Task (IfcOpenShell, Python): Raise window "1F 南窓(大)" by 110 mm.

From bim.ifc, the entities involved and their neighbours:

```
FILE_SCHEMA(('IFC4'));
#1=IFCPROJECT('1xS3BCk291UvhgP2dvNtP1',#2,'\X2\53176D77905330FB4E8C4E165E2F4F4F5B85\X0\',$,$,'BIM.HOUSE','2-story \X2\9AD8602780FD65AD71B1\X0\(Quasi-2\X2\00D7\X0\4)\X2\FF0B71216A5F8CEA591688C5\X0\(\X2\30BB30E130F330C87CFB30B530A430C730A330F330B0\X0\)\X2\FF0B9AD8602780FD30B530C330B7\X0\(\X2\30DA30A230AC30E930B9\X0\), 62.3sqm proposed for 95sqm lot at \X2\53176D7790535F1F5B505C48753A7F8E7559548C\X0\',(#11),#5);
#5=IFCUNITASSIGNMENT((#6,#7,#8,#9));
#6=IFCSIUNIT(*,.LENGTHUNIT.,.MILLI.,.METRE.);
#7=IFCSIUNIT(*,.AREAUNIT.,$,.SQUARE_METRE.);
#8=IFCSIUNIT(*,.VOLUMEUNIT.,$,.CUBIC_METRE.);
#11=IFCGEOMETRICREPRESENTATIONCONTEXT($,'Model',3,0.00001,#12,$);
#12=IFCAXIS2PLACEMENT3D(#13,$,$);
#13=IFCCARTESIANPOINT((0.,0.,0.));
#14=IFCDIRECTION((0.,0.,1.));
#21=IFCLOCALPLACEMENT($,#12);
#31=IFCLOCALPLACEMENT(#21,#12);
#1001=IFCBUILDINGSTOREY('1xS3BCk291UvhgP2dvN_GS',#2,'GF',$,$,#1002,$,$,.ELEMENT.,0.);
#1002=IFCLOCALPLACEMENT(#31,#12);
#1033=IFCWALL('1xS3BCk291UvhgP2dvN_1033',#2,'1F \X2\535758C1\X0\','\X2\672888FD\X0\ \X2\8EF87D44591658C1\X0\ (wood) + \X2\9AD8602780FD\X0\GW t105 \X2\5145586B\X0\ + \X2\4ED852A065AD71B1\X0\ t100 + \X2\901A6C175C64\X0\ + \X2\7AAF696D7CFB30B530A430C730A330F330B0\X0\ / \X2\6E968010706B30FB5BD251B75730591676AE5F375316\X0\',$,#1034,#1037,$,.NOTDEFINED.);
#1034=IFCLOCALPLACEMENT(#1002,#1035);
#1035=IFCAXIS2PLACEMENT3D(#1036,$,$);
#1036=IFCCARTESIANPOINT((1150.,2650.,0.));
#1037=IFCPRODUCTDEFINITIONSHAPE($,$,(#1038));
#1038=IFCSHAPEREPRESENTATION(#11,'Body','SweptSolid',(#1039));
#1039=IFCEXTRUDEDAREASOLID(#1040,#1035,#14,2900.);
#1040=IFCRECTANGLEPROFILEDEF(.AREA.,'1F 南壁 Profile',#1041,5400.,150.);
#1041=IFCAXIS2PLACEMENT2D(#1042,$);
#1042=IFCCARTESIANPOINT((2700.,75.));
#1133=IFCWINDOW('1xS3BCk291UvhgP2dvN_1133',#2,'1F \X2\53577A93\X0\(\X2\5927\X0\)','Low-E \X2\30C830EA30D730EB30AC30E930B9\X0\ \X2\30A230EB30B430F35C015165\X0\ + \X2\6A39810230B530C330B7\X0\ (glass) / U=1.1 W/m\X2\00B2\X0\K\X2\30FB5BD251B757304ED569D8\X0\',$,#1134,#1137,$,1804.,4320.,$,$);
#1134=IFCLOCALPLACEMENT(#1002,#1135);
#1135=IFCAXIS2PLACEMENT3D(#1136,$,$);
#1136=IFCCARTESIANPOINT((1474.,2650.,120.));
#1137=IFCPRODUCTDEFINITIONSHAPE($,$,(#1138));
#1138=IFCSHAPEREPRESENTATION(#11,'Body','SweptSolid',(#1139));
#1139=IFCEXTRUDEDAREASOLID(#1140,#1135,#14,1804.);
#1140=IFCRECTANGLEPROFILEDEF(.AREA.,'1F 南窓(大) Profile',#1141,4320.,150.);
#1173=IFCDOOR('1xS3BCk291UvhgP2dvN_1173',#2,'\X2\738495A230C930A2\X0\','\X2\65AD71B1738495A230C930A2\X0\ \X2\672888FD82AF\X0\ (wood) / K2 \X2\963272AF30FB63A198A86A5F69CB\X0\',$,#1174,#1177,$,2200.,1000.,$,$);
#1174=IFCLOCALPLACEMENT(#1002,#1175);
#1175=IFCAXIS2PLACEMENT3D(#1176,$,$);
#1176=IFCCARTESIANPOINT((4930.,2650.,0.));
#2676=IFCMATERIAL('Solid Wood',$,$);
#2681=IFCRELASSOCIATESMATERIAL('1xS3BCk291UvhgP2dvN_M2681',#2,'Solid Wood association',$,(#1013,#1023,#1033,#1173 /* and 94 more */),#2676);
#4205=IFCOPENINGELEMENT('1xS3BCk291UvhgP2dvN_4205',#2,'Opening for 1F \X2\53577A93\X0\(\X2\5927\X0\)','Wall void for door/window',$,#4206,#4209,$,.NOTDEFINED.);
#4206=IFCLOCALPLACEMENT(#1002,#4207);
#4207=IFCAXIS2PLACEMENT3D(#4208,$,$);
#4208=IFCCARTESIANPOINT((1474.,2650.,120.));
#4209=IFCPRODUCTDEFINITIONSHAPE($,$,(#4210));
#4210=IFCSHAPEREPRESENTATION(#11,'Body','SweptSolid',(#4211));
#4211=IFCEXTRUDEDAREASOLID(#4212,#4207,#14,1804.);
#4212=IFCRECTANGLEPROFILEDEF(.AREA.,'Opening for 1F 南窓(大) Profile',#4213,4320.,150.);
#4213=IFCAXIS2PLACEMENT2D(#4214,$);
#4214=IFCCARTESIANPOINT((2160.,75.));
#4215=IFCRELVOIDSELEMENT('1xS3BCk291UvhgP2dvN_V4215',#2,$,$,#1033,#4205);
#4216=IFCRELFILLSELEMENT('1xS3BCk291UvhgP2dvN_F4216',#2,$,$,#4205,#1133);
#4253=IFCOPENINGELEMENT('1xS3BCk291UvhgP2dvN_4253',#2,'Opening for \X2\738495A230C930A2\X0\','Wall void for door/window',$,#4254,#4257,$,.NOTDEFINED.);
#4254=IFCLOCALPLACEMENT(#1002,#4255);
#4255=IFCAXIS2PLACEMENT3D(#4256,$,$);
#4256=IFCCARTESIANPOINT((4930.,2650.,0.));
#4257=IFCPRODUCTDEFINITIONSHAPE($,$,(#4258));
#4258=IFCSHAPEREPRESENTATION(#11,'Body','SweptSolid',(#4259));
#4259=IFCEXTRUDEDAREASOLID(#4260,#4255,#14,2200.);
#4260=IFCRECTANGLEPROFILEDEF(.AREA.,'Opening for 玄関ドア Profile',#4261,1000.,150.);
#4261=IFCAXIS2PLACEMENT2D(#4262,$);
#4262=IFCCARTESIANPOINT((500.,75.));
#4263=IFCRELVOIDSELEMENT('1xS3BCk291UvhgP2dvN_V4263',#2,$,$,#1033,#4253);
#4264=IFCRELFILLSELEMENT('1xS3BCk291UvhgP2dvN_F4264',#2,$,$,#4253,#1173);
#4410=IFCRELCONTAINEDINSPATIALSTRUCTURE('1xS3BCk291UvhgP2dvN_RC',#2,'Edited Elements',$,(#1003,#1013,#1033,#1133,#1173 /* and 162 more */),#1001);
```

```python
import numpy as np
import ifcopenshell
import ifcopenshell.api.geometry
import ifcopenshell.util.placement
import ifcopenshell.util.unit

model = ifcopenshell.open("bim.ifc")
unit_scale = ifcopenshell.util.unit.calculate_unit_scale(model)

window = model.by_guid("1xS3BCk291UvhgP2dvN_1133")
opening = window.FillsVoids[0].RelatingOpeningElement
dz = 0.11 / unit_scale

shift = np.array([0.0, 0.0, dz])
# The window is not placed relative to its opening, so move both.
for product in (opening, window):
    matrix = ifcopenshell.util.placement.get_local_placement(product.ObjectPlacement)
    matrix[:3, 3] += shift
    ifcopenshell.api.geometry.edit_object_placement(model, product=product, matrix=matrix, is_si=False)

print(f"moved by {dz * unit_scale:+.3f} m")

model.write("bim_edited.ifc")
```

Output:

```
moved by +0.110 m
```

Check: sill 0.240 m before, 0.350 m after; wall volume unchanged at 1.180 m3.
